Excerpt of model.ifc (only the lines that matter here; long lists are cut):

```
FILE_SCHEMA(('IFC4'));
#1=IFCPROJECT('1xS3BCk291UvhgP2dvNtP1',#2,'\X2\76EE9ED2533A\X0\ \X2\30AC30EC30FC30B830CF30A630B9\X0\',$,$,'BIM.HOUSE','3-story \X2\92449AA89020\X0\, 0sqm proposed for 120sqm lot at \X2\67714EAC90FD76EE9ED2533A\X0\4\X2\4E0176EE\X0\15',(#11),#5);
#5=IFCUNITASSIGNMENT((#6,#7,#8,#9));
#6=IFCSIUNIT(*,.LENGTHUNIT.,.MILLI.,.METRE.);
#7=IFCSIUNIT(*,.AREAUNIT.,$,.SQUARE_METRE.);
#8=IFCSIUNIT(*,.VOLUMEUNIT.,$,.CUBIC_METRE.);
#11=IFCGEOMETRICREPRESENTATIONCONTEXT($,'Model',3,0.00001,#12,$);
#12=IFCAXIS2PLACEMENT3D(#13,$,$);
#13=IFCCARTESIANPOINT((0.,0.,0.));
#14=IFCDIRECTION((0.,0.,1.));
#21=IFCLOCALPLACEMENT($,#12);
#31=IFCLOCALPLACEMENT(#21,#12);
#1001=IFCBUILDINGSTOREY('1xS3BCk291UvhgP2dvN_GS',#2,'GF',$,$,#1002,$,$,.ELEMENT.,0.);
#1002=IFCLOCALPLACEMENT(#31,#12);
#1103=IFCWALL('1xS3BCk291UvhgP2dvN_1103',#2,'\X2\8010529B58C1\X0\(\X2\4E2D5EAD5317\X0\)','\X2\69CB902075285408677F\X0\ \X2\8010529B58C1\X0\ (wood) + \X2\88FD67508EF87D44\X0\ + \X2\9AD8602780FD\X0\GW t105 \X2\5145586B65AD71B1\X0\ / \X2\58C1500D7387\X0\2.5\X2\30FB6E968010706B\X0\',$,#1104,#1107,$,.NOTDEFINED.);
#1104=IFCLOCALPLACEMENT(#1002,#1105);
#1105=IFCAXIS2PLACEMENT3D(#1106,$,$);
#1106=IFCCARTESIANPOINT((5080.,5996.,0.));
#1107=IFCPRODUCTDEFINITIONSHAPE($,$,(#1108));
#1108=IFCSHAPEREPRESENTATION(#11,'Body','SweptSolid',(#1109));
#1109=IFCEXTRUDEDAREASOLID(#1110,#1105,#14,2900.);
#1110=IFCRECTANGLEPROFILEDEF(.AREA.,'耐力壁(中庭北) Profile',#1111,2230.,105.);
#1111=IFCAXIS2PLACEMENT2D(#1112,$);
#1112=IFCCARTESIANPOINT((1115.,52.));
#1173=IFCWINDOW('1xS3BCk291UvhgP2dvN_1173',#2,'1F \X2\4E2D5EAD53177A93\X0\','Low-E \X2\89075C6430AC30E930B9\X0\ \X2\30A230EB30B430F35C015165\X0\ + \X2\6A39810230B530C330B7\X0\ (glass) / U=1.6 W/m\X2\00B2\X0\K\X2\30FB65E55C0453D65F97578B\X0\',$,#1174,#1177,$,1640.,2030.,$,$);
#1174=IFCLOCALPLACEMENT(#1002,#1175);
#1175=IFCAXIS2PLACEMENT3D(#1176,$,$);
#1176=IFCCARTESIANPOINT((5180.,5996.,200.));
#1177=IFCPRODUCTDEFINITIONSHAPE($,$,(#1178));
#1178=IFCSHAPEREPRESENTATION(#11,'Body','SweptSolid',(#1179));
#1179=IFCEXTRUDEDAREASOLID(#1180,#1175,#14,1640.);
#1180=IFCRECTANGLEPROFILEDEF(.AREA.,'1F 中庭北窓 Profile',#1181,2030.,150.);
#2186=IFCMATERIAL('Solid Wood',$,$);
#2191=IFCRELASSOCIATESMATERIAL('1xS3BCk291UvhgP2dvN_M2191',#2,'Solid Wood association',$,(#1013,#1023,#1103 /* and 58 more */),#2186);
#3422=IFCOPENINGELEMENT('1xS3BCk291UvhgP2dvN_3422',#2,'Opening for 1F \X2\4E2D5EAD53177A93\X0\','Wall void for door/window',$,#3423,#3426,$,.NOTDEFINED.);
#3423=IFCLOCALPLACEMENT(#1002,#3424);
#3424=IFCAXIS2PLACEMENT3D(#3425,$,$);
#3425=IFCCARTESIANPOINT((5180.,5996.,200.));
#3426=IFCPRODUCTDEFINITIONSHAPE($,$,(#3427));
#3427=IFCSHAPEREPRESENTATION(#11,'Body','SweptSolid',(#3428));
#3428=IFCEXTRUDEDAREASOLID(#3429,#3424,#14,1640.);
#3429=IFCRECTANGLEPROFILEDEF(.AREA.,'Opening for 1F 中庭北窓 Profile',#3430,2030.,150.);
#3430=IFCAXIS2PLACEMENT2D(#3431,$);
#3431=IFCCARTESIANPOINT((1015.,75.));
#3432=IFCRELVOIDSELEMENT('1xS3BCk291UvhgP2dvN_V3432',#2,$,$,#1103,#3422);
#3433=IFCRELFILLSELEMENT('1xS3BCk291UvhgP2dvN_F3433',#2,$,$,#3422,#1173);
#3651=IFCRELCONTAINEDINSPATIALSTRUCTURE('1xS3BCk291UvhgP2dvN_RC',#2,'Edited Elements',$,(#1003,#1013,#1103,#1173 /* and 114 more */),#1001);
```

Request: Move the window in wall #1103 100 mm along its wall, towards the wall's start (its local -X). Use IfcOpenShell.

```python
import ifcopenshell
import ifcopenshell.api.geometry
import ifcopenshell.util.placement

model = ifcopenshell.open("model.ifc")

window = model.by_id(1173)
opening = window.FillsVoids[0].RelatingOpeningElement
wall = opening.VoidsElements[0].RelatingBuildingElement

wall_matrix = ifcopenshell.util.placement.get_local_placement(wall.ObjectPlacement)
shift = wall_matrix[:3, 0] * -100.0
before = ifcopenshell.util.placement.get_local_placement(window.ObjectPlacement)[:3, 3].copy()

# The window is not placed relative to its opening, so move both.
for product in (opening, window):
    matrix = ifcopenshell.util.placement.get_local_placement(product.ObjectPlacement)
    matrix[:3, 3] += shift
    ifcopenshell.api.geometry.edit_object_placement(model, product=product, matrix=matrix, is_si=False)

after = ifcopenshell.util.placement.get_local_placement(window.ObjectPlacement)[:3, 3]
print("window moved by", (after - before).round(3) + 0.0)

model.write("model_updated.ifc")
```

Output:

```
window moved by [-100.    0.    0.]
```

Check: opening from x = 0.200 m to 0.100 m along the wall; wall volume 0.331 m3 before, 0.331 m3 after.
